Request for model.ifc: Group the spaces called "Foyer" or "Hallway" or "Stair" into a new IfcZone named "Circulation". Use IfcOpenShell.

First a look at what the model holds.

```python
import ifcopenshell

model = ifcopenshell.open("model.ifc")
print(model.schema)
seen = {}
for space in model.by_type("IfcSpace"):
    seen[space.LongName] = seen.get(space.LongName, 0) + 1
for name, count in sorted(seen.items(), key=str):
    print(count, "x", name)
print("zones:", [z.Name for z in model.by_type("IfcZone")][:20])
```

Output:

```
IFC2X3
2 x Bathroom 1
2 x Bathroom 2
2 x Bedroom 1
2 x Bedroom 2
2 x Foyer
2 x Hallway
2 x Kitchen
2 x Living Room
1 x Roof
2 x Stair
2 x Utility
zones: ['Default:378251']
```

```python
import ifcopenshell
import ifcopenshell.api.group
import ifcopenshell.api.root

model = ifcopenshell.open("model.ifc")

names = {"Foyer", "Hallway", "Stair"}
spaces = [s for s in model.by_type("IfcSpace") if s.LongName in names]

zone = ifcopenshell.api.root.create_entity(model, ifc_class="IfcZone", name="Circulation")
ifcopenshell.api.group.assign_group(model, products=spaces, group=zone)
print(len(spaces), "spaces in", zone.Name)

model.write("model_updated.ifc")
```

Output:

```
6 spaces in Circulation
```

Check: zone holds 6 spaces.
